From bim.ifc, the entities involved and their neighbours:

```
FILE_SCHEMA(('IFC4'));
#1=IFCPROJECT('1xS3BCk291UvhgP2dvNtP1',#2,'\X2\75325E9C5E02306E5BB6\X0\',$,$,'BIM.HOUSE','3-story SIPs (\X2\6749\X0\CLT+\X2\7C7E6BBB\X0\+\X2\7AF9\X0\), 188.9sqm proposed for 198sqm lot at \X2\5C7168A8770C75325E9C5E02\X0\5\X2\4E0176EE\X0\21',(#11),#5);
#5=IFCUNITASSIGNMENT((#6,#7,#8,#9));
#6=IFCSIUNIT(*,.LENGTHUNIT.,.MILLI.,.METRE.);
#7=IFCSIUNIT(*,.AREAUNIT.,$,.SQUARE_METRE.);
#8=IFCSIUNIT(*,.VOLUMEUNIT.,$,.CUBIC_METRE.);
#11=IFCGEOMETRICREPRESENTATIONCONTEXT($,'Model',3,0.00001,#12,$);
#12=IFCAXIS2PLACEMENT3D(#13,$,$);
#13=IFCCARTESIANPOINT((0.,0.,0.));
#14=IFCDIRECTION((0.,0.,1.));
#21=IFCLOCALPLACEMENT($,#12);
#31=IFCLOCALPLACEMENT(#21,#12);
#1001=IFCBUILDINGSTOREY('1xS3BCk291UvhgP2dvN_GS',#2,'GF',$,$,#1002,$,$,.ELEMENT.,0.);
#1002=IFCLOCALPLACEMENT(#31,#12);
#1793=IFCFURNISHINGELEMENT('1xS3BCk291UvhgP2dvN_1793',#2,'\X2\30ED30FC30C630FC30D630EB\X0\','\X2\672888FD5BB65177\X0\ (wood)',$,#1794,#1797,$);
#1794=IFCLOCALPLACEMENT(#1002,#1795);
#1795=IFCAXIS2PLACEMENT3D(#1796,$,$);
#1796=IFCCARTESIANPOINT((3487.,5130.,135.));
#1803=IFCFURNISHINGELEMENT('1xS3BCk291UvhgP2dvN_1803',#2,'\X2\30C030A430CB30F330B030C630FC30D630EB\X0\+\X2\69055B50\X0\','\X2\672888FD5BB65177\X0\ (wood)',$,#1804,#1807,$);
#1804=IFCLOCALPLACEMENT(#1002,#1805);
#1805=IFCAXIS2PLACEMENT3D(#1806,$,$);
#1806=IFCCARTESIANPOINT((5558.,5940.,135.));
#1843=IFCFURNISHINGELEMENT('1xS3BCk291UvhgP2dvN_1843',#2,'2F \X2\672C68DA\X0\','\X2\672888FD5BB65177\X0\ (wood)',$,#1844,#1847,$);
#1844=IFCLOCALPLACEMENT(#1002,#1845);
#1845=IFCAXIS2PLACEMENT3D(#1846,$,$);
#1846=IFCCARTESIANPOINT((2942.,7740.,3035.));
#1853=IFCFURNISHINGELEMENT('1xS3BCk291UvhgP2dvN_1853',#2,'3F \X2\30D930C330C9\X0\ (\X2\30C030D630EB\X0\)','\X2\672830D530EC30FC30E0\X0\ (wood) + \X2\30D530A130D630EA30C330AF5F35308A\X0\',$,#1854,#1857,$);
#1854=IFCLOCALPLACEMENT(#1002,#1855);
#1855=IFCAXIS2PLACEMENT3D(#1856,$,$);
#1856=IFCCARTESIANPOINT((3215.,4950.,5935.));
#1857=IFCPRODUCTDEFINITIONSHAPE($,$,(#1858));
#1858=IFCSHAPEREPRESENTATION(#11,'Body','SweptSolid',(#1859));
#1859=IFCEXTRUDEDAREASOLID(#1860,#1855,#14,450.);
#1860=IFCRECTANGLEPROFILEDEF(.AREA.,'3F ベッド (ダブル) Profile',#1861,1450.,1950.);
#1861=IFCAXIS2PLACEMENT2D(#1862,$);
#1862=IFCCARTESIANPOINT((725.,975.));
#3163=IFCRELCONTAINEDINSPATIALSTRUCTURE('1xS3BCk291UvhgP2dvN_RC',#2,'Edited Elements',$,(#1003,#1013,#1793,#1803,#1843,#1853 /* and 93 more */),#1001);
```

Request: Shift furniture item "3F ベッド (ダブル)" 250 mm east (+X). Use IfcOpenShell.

```python
import ifcopenshell
import ifcopenshell.api.geometry
import ifcopenshell.util.placement

model = ifcopenshell.open("bim.ifc")

item = model.by_id(1853)
matrix = ifcopenshell.util.placement.get_local_placement(item.ObjectPlacement)
matrix[0, 3] += 250.0
ifcopenshell.api.geometry.edit_object_placement(model, product=item, matrix=matrix, is_si=False)

print(ifcopenshell.util.placement.get_local_placement(item.ObjectPlacement).round(3) + 0.0)

model.write("bim_updated.ifc")
```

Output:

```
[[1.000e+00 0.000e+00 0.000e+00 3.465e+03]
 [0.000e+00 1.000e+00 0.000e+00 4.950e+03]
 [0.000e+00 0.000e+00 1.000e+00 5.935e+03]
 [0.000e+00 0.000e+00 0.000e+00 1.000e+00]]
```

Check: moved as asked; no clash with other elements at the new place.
